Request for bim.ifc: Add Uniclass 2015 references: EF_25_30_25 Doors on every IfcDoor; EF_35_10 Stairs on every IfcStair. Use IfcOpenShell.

First a look at what the model holds.

```python
import ifcopenshell

model = ifcopenshell.open("bim.ifc")
print(model.schema)
print("classifications:", [c.Name for c in model.by_type("IfcClassification")])
for ifc_class in ("IfcDoor", "IfcRoof", "IfcStair", "IfcWall", "IfcWindow"):
    print(ifc_class, len(model.by_type(ifc_class)))
```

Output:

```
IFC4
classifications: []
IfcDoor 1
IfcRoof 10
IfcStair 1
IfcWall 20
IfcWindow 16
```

```python
import ifcopenshell
import ifcopenshell.api.classification

model = ifcopenshell.open("bim.ifc")

system = ifcopenshell.api.classification.add_classification(model, classification="Uniclass 2015")

codes = {
    "IfcDoor": ("EF_25_30_25", "Doors"),
    "IfcStair": ("EF_35_10", "Stairs"),
}
for ifc_class, (code, name) in codes.items():
    products = model.by_type(ifc_class)
    ifcopenshell.api.classification.add_reference(
        model, products=products, classification=system, identification=code, name=name
    )
    print(code, len(products))

model.write("bim_updated.ifc")
```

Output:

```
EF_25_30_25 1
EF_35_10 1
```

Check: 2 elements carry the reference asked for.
